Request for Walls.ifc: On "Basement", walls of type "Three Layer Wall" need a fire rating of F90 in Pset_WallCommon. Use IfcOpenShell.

First a look at what the model holds.

```python
import ifcopenshell
import ifcopenshell.util.element

model = ifcopenshell.open("Walls.ifc")
print(model.schema)
storey = next(s for s in model.by_type("IfcBuildingStorey") if s.Name == "Basement")
walls = [e for e in ifcopenshell.util.element.get_decomposition(storey) if e.is_a("IfcWall")]
seen = {}
for e in walls:
    element_type = ifcopenshell.util.element.get_type(e)
    key = (element_type.Name if element_type != e and element_type else None, ifcopenshell.util.element.get_pset(e, "Pset_WallCommon", "FireRating"))
    seen[key] = seen.get(key, 0) + 1
for (name, value), count in sorted(seen.items(), key=str):
    print(count, "x", name, "|", value)
```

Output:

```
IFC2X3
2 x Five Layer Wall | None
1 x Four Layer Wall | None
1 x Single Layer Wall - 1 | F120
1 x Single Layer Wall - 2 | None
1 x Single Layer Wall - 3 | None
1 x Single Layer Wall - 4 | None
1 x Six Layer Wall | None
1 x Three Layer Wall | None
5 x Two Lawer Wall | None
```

```python
import ifcopenshell
import ifcopenshell.api.pset
import ifcopenshell.util.element

model = ifcopenshell.open("Walls.ifc")

storey = next(s for s in model.by_type("IfcBuildingStorey") if s.Name == "Basement")
walls = [e for e in ifcopenshell.util.element.get_decomposition(storey) if e.is_a("IfcWall")]

count = 0
for e in walls:
    element_type = ifcopenshell.util.element.get_type(e)
    if element_type in (None, e) or element_type.Name != "Three Layer Wall":
        continue
    # add_pset returns the element's existing set when there is one.
    pset = ifcopenshell.api.pset.add_pset(model, product=e, name="Pset_WallCommon")
    ifcopenshell.api.pset.edit_pset(model, pset=pset, properties={"FireRating": "F90"})
    count += 1

print(count, "walls updated")

model.write("Walls-out.ifc")
```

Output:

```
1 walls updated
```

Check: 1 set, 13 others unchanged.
